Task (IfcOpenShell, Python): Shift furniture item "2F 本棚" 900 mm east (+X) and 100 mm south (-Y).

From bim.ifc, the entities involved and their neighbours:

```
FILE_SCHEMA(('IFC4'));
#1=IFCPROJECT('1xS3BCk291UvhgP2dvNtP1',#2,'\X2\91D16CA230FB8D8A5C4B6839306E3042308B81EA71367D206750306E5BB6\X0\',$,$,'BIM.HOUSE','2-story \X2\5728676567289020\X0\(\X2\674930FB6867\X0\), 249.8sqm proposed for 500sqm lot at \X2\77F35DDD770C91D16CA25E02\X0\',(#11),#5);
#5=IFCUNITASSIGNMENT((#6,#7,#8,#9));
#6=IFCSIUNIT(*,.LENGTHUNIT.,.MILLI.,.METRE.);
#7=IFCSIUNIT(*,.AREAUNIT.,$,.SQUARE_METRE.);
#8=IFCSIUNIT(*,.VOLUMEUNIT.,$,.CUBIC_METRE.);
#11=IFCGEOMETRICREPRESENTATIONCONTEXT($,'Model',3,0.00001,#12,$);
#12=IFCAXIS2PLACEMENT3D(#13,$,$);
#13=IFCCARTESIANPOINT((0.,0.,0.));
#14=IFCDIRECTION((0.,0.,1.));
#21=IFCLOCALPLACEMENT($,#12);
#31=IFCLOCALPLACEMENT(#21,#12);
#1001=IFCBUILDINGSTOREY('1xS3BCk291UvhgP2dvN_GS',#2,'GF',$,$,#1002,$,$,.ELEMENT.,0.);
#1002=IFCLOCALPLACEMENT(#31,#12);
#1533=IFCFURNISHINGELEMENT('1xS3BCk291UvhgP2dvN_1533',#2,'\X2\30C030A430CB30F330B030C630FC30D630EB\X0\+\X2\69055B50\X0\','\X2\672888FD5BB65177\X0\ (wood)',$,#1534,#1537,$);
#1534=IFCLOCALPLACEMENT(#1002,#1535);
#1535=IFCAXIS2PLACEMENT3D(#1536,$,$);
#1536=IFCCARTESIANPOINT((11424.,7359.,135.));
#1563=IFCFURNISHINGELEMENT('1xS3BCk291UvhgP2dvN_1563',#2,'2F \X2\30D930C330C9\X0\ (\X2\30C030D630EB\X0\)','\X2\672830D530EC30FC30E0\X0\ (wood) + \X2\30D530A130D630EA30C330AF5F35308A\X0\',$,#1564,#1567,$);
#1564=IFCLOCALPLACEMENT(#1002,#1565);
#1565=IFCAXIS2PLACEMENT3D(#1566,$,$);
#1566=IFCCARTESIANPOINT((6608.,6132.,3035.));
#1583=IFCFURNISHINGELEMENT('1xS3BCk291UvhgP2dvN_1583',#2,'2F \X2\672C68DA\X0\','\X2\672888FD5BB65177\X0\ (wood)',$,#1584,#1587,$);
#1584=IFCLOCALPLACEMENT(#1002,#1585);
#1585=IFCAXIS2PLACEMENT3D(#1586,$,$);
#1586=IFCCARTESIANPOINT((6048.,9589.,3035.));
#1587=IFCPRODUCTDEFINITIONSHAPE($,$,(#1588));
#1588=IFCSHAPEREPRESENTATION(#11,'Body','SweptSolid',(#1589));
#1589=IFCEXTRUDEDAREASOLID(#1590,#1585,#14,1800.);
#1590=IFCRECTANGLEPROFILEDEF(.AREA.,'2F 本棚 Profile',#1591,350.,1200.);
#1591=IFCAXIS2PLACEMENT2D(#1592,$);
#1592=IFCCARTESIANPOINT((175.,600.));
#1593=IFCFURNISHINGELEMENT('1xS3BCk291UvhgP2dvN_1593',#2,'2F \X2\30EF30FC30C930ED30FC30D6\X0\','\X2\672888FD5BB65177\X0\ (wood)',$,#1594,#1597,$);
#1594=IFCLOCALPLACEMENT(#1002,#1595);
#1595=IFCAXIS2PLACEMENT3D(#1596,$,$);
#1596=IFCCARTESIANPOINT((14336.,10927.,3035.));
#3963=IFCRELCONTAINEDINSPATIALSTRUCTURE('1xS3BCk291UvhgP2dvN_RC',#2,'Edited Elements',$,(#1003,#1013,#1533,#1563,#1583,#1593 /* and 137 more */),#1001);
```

```python
import ifcopenshell
import ifcopenshell.api.geometry
import ifcopenshell.util.placement
import ifcopenshell.util.unit

model = ifcopenshell.open("bim.ifc")
unit_scale = ifcopenshell.util.unit.calculate_unit_scale(model)

item = model.by_id(1583)
matrix = ifcopenshell.util.placement.get_local_placement(item.ObjectPlacement)
matrix[0, 3] += 0.9 / unit_scale
matrix[1, 3] -= 0.1 / unit_scale
ifcopenshell.api.geometry.edit_object_placement(model, product=item, matrix=matrix, is_si=False)

print(ifcopenshell.util.placement.get_local_placement(item.ObjectPlacement).round(3) + 0.0)

model.write("bim-out.ifc")
```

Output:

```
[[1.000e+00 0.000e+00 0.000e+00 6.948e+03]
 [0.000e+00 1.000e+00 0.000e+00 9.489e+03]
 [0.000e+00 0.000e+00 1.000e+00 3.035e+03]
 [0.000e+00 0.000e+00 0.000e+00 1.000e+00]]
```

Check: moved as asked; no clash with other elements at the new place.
